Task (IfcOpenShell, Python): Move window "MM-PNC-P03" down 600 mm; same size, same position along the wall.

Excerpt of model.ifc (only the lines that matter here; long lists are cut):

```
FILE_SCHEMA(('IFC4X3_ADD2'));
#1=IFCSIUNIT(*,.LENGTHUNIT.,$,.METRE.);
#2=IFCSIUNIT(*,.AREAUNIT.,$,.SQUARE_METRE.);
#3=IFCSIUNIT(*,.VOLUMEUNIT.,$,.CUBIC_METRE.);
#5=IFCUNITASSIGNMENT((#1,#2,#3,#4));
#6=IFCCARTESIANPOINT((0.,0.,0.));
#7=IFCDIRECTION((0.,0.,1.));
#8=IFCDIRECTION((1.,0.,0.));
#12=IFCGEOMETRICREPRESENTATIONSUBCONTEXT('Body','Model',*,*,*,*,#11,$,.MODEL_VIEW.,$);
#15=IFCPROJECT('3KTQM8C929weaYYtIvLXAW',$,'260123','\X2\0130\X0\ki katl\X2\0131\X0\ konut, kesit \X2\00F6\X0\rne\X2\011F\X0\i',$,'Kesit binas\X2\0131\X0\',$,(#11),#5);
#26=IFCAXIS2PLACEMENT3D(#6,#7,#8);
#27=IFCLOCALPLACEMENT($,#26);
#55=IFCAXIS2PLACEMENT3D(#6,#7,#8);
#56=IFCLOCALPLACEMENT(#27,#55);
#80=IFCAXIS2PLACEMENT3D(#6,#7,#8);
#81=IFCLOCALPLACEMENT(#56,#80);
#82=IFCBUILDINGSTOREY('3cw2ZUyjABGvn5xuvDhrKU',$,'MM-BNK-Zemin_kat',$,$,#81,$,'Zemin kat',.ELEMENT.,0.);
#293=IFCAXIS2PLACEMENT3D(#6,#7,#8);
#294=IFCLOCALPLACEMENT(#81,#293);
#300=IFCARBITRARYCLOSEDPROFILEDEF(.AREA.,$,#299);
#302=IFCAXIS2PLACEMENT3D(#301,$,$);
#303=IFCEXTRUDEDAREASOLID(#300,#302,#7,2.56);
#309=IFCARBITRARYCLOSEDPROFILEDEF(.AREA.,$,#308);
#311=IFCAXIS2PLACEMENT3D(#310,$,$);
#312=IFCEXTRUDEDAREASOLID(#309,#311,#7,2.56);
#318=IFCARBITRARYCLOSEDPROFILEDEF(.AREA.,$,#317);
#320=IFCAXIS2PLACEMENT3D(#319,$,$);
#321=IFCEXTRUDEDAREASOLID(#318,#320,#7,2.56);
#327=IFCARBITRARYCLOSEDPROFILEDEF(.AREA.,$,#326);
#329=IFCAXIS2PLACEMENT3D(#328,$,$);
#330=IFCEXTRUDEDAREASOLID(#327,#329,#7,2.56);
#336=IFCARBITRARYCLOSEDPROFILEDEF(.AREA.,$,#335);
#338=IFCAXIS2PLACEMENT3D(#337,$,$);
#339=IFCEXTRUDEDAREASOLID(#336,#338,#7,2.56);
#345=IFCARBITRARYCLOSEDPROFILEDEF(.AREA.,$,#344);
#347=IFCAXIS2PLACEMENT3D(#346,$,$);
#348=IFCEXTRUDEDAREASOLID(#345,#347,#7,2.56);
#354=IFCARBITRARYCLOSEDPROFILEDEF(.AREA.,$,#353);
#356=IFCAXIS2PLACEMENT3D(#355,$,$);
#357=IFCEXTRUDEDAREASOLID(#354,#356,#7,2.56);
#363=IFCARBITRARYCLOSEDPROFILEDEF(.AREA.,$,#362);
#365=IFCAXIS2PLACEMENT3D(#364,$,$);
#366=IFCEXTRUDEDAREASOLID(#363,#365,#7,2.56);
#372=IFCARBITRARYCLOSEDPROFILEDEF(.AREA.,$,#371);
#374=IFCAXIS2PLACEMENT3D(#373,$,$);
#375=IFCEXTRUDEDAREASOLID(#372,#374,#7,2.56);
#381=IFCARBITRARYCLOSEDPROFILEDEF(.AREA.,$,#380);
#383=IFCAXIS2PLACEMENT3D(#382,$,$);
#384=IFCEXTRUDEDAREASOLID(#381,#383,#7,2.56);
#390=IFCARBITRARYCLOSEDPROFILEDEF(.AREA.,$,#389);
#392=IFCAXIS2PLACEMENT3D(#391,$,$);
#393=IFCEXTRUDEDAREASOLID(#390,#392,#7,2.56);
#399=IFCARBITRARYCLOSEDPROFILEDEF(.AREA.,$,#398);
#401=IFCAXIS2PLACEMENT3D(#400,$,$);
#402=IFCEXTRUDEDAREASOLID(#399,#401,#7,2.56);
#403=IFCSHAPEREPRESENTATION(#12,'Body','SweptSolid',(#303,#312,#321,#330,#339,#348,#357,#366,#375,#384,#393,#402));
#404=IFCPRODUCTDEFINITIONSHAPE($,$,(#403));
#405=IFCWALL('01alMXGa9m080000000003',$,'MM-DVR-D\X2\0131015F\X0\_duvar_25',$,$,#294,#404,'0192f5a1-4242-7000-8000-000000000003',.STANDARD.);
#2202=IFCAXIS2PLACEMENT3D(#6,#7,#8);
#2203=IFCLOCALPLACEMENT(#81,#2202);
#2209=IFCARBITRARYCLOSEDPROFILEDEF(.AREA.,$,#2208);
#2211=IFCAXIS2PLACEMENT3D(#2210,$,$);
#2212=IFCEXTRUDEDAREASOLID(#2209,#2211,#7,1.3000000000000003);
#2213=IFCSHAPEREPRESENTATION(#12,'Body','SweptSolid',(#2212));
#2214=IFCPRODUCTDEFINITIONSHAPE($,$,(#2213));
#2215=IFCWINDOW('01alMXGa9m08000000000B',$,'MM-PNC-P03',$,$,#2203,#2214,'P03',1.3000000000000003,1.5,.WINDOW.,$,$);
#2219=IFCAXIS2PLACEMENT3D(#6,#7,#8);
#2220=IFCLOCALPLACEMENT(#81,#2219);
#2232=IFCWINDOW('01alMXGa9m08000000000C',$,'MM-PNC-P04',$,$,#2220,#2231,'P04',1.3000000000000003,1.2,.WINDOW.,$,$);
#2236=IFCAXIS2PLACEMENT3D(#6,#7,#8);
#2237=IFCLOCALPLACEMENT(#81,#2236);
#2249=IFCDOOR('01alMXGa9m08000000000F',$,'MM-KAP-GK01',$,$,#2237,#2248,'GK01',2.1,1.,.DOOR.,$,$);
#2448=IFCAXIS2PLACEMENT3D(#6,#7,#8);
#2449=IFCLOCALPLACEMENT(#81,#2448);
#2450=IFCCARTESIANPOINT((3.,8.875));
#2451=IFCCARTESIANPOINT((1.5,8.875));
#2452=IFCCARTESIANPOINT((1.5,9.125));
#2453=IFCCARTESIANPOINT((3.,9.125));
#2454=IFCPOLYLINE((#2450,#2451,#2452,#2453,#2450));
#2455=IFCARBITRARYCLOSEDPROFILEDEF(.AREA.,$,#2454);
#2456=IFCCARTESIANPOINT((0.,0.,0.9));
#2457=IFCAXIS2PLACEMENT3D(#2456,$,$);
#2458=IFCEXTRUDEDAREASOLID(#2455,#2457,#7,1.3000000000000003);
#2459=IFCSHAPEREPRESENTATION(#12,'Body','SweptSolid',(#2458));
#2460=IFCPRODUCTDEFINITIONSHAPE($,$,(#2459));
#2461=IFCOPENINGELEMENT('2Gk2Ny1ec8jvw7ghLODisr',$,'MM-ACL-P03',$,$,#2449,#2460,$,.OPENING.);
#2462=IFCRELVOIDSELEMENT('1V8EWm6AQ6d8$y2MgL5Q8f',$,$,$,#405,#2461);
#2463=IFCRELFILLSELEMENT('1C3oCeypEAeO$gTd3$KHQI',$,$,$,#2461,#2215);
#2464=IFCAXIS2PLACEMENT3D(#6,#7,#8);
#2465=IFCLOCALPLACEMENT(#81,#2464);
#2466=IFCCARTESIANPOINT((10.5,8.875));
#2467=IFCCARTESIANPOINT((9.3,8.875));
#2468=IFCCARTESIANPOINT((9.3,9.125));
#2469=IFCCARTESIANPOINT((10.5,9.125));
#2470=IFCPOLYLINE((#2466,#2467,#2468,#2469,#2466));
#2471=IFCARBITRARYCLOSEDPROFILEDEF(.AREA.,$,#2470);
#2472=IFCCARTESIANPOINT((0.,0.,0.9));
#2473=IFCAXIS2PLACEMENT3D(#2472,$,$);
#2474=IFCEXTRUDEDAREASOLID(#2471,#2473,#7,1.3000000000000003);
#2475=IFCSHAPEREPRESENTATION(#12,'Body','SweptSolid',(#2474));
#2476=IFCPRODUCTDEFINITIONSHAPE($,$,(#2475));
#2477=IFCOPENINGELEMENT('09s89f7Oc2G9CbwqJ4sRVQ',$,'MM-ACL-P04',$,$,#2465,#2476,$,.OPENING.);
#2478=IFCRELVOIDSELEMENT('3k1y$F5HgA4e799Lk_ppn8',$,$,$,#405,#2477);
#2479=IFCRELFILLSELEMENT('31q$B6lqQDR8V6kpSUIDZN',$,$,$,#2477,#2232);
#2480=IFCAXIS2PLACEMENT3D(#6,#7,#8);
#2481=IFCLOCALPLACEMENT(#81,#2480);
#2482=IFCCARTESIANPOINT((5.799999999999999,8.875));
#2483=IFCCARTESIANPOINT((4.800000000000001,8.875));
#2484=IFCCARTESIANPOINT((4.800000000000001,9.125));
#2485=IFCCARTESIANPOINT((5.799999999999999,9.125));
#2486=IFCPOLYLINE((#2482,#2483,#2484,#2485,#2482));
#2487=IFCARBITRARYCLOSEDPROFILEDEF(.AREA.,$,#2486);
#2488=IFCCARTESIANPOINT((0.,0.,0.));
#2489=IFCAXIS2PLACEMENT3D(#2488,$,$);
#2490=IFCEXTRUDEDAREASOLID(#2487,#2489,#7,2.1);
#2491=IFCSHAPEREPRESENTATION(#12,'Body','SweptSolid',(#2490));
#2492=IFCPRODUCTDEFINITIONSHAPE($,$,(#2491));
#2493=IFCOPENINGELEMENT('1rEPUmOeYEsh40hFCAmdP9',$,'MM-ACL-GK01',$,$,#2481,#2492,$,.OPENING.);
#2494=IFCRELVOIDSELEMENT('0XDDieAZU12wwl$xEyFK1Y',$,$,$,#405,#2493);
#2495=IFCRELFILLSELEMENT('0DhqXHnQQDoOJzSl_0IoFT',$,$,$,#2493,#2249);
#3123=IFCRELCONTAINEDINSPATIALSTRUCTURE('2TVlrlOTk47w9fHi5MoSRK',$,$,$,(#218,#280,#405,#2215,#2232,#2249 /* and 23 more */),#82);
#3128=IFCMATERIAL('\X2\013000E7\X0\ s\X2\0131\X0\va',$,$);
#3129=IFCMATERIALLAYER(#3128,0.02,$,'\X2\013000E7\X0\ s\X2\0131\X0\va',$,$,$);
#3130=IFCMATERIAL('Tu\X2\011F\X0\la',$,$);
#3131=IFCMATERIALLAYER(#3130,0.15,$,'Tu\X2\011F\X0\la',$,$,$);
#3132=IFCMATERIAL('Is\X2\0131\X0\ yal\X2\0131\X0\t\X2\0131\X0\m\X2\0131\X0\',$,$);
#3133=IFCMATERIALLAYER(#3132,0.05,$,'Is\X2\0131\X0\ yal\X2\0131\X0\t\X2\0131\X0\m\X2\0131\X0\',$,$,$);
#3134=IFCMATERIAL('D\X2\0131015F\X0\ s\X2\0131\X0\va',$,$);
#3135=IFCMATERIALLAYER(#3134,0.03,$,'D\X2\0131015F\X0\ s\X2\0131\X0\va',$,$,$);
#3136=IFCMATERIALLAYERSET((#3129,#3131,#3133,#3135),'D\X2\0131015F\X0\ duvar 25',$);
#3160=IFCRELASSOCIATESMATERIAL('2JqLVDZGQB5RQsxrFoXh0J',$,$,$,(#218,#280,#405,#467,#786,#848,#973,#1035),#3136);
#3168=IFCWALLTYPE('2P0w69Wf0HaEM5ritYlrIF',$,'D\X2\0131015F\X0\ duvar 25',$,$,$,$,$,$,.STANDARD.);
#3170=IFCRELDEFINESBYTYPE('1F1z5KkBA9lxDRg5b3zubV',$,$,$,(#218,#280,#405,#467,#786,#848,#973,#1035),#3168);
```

```python
import numpy as np
import ifcopenshell
import ifcopenshell.api.geometry
import ifcopenshell.util.placement
import ifcopenshell.util.unit

model = ifcopenshell.open("model.ifc")
unit_scale = ifcopenshell.util.unit.calculate_unit_scale(model)

window = model.by_id(2215)
opening = window.FillsVoids[0].RelatingOpeningElement
dz = -0.6 / unit_scale

shift = np.array([0.0, 0.0, dz])
# The window is not placed relative to its opening, so move both.
for product in (opening, window):
    matrix = ifcopenshell.util.placement.get_local_placement(product.ObjectPlacement)
    matrix[:3, 3] += shift
    ifcopenshell.api.geometry.edit_object_placement(model, product=product, matrix=matrix, is_si=False)

print(f"moved by {dz * unit_scale:+.3f} m")

model.write("model_v2.ifc")
```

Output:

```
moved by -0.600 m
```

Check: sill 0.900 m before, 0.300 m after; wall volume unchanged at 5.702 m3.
